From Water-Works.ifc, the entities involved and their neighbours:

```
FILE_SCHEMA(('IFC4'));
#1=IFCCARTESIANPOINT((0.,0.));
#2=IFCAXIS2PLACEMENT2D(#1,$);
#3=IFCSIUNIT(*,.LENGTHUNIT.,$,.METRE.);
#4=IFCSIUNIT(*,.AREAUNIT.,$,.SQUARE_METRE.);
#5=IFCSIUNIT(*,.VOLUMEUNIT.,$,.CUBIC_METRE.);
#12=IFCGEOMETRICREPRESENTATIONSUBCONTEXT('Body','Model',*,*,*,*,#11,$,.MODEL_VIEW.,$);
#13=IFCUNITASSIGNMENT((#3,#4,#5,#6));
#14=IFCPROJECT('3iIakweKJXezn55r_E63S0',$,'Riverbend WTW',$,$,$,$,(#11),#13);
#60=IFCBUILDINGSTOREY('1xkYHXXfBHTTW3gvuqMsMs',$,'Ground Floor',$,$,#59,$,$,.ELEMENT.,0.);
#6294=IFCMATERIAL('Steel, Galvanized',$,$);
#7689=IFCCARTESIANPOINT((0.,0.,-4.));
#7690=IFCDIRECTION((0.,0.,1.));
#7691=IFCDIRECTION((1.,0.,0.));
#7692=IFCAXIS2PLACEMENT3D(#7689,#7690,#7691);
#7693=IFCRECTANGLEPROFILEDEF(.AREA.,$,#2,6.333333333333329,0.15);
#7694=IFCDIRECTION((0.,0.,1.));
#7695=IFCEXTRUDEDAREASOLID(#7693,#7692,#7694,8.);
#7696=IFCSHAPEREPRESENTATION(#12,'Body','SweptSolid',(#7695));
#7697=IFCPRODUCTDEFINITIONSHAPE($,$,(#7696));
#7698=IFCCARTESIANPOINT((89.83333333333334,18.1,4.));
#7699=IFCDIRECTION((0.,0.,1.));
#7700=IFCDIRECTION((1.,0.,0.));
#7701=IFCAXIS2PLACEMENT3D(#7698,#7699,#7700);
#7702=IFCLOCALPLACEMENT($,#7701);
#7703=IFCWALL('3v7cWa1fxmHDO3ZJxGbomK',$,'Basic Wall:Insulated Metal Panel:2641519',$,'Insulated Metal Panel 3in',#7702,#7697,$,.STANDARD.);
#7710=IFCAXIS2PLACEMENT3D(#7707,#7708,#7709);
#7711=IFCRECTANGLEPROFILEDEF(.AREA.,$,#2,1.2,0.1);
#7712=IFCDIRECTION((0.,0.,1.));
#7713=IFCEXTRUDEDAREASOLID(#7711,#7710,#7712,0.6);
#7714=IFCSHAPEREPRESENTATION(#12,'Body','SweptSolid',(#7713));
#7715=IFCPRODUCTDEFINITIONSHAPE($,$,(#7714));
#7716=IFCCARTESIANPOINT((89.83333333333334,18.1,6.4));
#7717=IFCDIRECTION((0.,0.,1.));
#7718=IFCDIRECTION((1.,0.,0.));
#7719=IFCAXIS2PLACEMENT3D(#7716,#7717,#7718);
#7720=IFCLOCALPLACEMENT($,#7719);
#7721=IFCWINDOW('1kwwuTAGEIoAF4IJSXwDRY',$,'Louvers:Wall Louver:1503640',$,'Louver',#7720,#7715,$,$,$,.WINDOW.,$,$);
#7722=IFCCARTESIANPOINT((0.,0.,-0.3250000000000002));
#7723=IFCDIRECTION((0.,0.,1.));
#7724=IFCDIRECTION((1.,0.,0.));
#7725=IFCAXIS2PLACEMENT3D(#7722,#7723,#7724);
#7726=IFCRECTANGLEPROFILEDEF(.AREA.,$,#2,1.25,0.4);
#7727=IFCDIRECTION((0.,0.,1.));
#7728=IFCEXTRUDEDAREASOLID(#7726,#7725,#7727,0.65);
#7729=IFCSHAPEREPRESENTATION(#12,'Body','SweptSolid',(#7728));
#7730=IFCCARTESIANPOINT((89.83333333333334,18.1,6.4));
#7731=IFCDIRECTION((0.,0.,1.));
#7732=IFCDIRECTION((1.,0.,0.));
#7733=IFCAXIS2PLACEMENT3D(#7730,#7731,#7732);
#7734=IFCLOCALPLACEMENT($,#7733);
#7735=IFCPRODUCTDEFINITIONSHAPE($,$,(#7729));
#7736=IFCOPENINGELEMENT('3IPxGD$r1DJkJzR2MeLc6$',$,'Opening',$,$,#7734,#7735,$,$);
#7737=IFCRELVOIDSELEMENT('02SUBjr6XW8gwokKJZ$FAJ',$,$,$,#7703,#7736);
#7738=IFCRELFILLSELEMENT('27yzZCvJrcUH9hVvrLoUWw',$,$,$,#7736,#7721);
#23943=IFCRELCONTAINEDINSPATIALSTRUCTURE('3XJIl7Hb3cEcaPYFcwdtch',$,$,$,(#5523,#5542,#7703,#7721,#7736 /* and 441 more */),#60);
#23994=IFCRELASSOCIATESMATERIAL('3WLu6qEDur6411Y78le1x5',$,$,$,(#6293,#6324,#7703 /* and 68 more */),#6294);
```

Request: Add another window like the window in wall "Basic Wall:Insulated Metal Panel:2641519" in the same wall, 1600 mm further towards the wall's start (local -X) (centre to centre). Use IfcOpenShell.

```python
import ifcopenshell
import ifcopenshell.api.feature
import ifcopenshell.api.geometry
import ifcopenshell.api.root
import ifcopenshell.geom
import ifcopenshell.util.element
import ifcopenshell.util.placement
import ifcopenshell.util.shape
import ifcopenshell.util.unit

model = ifcopenshell.open("Water-Works.ifc")
unit_scale = ifcopenshell.util.unit.calculate_unit_scale(model)
settings = ifcopenshell.geom.settings()


def volume(element):
    """Net volume in cubic metres, openings subtracted."""
    shape = ifcopenshell.geom.create_shape(settings, element)
    return ifcopenshell.util.shape.get_volume(shape.geometry)


window = model.by_guid("1kwwuTAGEIoAF4IJSXwDRY")
opening = window.FillsVoids[0].RelatingOpeningElement
wall = opening.VoidsElements[0].RelatingBuildingElement
before = volume(wall)
shift = ifcopenshell.util.placement.get_local_placement(wall.ObjectPlacement)[:3, 0] * -1.6 / unit_scale

# copy_class copies the void relationship, type, container and properties, but no geometry.
new_opening = ifcopenshell.api.root.copy_class(model, product=opening)
new_opening.Representation = ifcopenshell.util.element.copy_deep(
    model, opening.Representation, exclude=["IfcGeometricRepresentationContext", "IfcRepresentationMap"]
)
new_window = ifcopenshell.api.root.copy_class(model, product=window)
new_window.Representation = ifcopenshell.util.element.copy_deep(
    model, window.Representation, exclude=["IfcGeometricRepresentationContext", "IfcRepresentationMap"]
)
new_window.Name = "Louvers:Wall Louver"
ifcopenshell.api.feature.add_filling(model, opening=new_opening, element=new_window)

for old, new in ((opening, new_opening), (window, new_window)):
    matrix = ifcopenshell.util.placement.get_local_placement(old.ObjectPlacement)
    matrix[:3, 3] += shift
    ifcopenshell.api.geometry.edit_object_placement(model, product=new, matrix=matrix, is_si=False)

after = volume(wall)

print(f"wall volume {before:.3f} -> {after:.3f} m3")

model.write("Water-Works_edited.ifc")
```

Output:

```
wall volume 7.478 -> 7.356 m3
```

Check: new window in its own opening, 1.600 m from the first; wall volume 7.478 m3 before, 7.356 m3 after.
